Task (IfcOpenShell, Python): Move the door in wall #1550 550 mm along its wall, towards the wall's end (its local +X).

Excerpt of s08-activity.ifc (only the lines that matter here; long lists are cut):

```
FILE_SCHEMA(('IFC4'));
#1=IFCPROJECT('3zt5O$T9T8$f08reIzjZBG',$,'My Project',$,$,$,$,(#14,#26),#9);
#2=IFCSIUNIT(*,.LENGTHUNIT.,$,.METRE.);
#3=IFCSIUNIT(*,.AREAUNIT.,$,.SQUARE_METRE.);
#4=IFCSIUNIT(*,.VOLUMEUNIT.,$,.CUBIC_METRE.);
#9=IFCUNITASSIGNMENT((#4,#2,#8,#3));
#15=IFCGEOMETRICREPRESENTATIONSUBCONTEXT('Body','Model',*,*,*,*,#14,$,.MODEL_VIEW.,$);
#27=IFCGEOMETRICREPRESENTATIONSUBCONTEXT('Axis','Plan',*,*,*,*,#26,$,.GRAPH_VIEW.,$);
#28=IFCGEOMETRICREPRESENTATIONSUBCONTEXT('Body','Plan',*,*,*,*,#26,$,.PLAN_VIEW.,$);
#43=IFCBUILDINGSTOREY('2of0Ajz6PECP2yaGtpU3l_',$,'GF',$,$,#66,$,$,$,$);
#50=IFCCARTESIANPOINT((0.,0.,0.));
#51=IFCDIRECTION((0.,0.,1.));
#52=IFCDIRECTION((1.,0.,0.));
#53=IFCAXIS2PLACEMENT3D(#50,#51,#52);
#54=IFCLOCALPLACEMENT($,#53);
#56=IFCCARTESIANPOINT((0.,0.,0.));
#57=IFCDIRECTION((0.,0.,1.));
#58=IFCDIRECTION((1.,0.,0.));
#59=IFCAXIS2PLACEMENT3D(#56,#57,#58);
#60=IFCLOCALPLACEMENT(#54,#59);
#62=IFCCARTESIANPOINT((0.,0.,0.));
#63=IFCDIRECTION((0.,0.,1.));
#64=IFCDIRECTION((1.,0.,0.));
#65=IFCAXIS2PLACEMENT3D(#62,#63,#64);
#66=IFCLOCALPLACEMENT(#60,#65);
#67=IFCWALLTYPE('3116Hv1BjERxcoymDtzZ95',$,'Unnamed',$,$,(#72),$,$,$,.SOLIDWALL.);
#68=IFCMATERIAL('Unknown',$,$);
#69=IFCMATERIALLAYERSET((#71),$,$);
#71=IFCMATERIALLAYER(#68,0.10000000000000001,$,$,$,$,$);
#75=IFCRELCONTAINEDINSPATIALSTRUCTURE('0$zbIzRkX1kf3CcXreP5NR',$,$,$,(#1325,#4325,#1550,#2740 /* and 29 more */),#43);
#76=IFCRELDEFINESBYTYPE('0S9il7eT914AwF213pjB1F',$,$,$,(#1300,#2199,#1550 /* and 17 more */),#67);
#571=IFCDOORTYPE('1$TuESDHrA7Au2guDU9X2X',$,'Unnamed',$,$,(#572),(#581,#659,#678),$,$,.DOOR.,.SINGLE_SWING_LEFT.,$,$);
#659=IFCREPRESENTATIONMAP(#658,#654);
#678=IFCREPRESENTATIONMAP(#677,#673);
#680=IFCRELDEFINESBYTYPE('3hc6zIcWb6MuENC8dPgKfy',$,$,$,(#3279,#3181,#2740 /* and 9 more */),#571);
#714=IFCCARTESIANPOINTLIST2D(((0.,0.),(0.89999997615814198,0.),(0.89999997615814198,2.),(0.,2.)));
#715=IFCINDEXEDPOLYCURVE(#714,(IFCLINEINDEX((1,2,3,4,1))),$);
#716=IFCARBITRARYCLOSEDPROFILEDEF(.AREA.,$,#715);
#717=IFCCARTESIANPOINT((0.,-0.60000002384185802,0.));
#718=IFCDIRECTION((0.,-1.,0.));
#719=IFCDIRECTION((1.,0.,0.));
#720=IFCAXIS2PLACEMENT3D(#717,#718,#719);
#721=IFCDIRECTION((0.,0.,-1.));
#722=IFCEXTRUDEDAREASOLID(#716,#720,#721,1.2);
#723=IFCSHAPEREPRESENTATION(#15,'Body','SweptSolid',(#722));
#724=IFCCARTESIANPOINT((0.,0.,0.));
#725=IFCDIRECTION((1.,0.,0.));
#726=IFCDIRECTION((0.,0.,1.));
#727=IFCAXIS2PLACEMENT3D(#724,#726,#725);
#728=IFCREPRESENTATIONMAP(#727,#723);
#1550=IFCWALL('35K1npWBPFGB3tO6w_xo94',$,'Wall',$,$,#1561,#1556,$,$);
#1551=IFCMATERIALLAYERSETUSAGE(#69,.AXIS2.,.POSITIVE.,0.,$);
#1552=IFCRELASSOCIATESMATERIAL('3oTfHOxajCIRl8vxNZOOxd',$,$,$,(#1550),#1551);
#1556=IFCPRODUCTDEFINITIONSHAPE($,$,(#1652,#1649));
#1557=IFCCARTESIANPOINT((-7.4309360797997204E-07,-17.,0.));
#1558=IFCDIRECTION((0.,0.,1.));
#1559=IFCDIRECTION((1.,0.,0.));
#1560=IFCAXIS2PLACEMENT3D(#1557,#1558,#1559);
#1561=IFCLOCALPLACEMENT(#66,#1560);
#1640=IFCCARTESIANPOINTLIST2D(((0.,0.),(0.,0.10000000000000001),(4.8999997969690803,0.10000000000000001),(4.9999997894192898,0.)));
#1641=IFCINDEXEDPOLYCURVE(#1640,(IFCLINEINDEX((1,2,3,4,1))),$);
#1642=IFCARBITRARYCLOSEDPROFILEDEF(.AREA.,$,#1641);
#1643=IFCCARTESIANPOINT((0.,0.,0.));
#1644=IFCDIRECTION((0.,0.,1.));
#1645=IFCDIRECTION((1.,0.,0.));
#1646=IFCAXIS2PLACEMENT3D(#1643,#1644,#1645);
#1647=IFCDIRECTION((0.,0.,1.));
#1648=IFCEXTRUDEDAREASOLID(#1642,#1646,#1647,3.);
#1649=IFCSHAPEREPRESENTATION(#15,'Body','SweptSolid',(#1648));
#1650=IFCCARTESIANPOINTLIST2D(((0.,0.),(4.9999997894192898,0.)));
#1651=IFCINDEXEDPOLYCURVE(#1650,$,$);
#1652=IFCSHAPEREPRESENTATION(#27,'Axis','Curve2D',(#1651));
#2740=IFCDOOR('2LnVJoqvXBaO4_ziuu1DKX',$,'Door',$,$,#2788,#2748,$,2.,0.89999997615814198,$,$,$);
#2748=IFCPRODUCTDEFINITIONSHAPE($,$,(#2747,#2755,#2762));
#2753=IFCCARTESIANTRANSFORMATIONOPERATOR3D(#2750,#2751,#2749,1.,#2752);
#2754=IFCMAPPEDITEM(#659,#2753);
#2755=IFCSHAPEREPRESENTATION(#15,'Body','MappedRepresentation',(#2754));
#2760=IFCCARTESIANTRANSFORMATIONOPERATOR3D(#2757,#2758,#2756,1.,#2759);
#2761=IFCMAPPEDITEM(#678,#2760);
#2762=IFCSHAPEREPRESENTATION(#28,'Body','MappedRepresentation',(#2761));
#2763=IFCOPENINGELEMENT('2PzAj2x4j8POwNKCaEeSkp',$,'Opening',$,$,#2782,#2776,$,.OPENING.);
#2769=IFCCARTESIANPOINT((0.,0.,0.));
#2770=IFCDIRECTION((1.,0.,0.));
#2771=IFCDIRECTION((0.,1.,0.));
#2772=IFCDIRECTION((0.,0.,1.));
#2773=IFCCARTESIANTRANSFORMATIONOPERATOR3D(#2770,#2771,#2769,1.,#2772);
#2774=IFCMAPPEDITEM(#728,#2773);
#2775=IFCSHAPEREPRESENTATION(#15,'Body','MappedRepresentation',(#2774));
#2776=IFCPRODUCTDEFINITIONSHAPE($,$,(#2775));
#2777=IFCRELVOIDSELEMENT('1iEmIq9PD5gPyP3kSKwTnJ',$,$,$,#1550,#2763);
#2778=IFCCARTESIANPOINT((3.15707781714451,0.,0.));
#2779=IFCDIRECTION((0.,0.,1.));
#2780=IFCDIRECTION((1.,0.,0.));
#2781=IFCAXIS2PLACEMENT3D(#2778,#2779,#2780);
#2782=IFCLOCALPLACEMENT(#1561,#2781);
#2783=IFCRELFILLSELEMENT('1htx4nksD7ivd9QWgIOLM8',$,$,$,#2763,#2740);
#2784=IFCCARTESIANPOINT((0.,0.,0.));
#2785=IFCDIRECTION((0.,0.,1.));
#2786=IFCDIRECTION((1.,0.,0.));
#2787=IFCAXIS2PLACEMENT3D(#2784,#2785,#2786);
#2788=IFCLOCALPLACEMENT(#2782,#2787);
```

```python
import ifcopenshell
import ifcopenshell.api.geometry
import ifcopenshell.util.placement
import ifcopenshell.util.unit

model = ifcopenshell.open("s08-activity.ifc")
unit_scale = ifcopenshell.util.unit.calculate_unit_scale(model)

door = model.by_guid("2LnVJoqvXBaO4_ziuu1DKX")
opening = door.FillsVoids[0].RelatingOpeningElement
wall = opening.VoidsElements[0].RelatingBuildingElement

wall_matrix = ifcopenshell.util.placement.get_local_placement(wall.ObjectPlacement)
shift = wall_matrix[:3, 0] * 0.55 / unit_scale
before = ifcopenshell.util.placement.get_local_placement(door.ObjectPlacement)[:3, 3].copy()

# The door is placed relative to its opening, so it follows when the opening moves.
matrix = ifcopenshell.util.placement.get_local_placement(opening.ObjectPlacement)
matrix[:3, 3] += shift
ifcopenshell.api.geometry.edit_object_placement(
    model, product=opening, matrix=matrix, is_si=False, should_transform_children=True
)

after = ifcopenshell.util.placement.get_local_placement(door.ObjectPlacement)[:3, 3]
print("door moved by", (after - before).round(3) + 0.0)

model.write("s08-activity_rev.ifc")
```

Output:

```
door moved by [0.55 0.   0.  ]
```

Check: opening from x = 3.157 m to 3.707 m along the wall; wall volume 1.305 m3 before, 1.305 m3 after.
